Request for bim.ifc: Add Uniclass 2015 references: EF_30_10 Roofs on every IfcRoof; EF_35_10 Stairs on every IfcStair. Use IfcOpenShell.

First a look at what the model holds.

```python
import ifcopenshell

model = ifcopenshell.open("bim.ifc")
print(model.schema)
print("classifications:", [c.Name for c in model.by_type("IfcClassification")])
for ifc_class in ("IfcDoor", "IfcRoof", "IfcStair", "IfcWall", "IfcWindow"):
    print(ifc_class, len(model.by_type(ifc_class)))
```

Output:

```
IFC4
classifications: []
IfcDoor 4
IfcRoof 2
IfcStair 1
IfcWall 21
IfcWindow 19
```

```python
import ifcopenshell
import ifcopenshell.api.classification

model = ifcopenshell.open("bim.ifc")

system = ifcopenshell.api.classification.add_classification(model, classification="Uniclass 2015")

codes = {
    "IfcRoof": ("EF_30_10", "Roofs"),
    "IfcStair": ("EF_35_10", "Stairs"),
}
for ifc_class, (code, name) in codes.items():
    products = model.by_type(ifc_class)
    ifcopenshell.api.classification.add_reference(
        model, products=products, classification=system, identification=code, name=name
    )
    print(code, len(products))

model.write("bim_rev.ifc")
```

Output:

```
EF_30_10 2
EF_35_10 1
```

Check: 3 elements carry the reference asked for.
